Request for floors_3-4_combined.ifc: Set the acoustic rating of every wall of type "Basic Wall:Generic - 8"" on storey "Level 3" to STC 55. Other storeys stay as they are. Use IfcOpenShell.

First a look at what the model holds.

```python
import ifcopenshell
import ifcopenshell.util.element

model = ifcopenshell.open("floors_3-4_combined.ifc")
print(model.schema)
storey = next(s for s in model.by_type("IfcBuildingStorey") if s.Name == "Level 3")
walls = [e for e in ifcopenshell.util.element.get_decomposition(storey) if e.is_a("IfcWall")]
seen = {}
for e in walls:
    element_type = ifcopenshell.util.element.get_type(e)
    key = (element_type.Name if element_type != e and element_type else None, ifcopenshell.util.element.get_pset(e, "Pset_WallCommon", "AcousticRating"))
    seen[key] = seen.get(key, 0) + 1
for (name, value), count in sorted(seen.items(), key=str):
    print(count, "x", name, "|", value)
```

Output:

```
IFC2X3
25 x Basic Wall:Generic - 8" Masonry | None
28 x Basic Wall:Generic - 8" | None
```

```python
import ifcopenshell
import ifcopenshell.api.pset
import ifcopenshell.util.element

model = ifcopenshell.open("floors_3-4_combined.ifc")

storey = next(s for s in model.by_type("IfcBuildingStorey") if s.Name == "Level 3")
walls = [e for e in ifcopenshell.util.element.get_decomposition(storey) if e.is_a("IfcWall")]

count = 0
for e in walls:
    element_type = ifcopenshell.util.element.get_type(e)
    if element_type in (None, e) or element_type.Name != 'Basic Wall:Generic - 8"':
        continue
    # add_pset returns the element's existing set when there is one.
    pset = ifcopenshell.api.pset.add_pset(model, product=e, name="Pset_WallCommon")
    ifcopenshell.api.pset.edit_pset(model, pset=pset, properties={"AcousticRating": "STC 55"})
    count += 1

print(count, "walls updated")

model.write("floors_3-4_combined-out.ifc")
```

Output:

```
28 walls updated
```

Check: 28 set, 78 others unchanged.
